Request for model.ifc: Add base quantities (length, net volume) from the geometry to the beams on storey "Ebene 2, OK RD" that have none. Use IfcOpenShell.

First a look at what the model holds.

```python
import ifcopenshell
import ifcopenshell.util.element
import ifcopenshell.util.unit

model = ifcopenshell.open("model.ifc")
print(model.schema)
for unit_type in ("LENGTHUNIT", "AREAUNIT", "VOLUMEUNIT"):
    print(unit_type, ifcopenshell.util.unit.calculate_unit_scale(model, unit_type))
storey = next(s for s in model.by_type("IfcBuildingStorey") if s.Name == "Ebene 2, OK RD")
beams = [e for e in ifcopenshell.util.element.get_decomposition(storey) if e.is_a("IfcBeam")]
for e in sorted(beams, key=lambda e: e.id()):
    print(e.id(), e.is_a(), e.Name, list(ifcopenshell.util.element.get_psets(e, qtos_only=True)), sep=" | ")
```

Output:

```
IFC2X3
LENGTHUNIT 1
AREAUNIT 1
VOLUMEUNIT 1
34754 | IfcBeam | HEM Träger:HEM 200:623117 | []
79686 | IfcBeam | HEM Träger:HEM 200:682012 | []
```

```python
import ifcopenshell
import ifcopenshell.api.pset
import ifcopenshell.geom
import ifcopenshell.util.element
import ifcopenshell.util.shape
import ifcopenshell.util.unit

model = ifcopenshell.open("model.ifc")
unit_scale = ifcopenshell.util.unit.calculate_unit_scale(model)
volume_scale = ifcopenshell.util.unit.calculate_unit_scale(model, "VOLUMEUNIT")
settings = ifcopenshell.geom.settings()

storey = next(s for s in model.by_type("IfcBuildingStorey") if s.Name == "Ebene 2, OK RD")
beams = [e for e in ifcopenshell.util.element.get_decomposition(storey) if e.is_a("IfcBeam")]

for e in sorted(beams, key=lambda e: e.id()):
    if ifcopenshell.util.element.get_psets(e, qtos_only=True, should_inherit=False):
        continue
    # Geometry comes back in metres, in the element's own axes.
    shape = ifcopenshell.geom.create_shape(settings, e)
    values = {
        "Length": ifcopenshell.util.shape.get_max_xyz(shape.geometry) / unit_scale,
        "NetVolume": ifcopenshell.util.shape.get_volume(shape.geometry) / volume_scale,
    }
    qto = ifcopenshell.api.pset.add_qto(model, product=e, name="BaseQuantities")
    ifcopenshell.api.pset.edit_qto(model, qto=qto, properties=values)
    print(e.id(), {k: round(v, 3) for k, v in values.items()})

model.write("model_updated.ifc")
```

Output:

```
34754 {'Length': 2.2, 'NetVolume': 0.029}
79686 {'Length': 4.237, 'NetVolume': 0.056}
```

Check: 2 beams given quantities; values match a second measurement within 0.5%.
